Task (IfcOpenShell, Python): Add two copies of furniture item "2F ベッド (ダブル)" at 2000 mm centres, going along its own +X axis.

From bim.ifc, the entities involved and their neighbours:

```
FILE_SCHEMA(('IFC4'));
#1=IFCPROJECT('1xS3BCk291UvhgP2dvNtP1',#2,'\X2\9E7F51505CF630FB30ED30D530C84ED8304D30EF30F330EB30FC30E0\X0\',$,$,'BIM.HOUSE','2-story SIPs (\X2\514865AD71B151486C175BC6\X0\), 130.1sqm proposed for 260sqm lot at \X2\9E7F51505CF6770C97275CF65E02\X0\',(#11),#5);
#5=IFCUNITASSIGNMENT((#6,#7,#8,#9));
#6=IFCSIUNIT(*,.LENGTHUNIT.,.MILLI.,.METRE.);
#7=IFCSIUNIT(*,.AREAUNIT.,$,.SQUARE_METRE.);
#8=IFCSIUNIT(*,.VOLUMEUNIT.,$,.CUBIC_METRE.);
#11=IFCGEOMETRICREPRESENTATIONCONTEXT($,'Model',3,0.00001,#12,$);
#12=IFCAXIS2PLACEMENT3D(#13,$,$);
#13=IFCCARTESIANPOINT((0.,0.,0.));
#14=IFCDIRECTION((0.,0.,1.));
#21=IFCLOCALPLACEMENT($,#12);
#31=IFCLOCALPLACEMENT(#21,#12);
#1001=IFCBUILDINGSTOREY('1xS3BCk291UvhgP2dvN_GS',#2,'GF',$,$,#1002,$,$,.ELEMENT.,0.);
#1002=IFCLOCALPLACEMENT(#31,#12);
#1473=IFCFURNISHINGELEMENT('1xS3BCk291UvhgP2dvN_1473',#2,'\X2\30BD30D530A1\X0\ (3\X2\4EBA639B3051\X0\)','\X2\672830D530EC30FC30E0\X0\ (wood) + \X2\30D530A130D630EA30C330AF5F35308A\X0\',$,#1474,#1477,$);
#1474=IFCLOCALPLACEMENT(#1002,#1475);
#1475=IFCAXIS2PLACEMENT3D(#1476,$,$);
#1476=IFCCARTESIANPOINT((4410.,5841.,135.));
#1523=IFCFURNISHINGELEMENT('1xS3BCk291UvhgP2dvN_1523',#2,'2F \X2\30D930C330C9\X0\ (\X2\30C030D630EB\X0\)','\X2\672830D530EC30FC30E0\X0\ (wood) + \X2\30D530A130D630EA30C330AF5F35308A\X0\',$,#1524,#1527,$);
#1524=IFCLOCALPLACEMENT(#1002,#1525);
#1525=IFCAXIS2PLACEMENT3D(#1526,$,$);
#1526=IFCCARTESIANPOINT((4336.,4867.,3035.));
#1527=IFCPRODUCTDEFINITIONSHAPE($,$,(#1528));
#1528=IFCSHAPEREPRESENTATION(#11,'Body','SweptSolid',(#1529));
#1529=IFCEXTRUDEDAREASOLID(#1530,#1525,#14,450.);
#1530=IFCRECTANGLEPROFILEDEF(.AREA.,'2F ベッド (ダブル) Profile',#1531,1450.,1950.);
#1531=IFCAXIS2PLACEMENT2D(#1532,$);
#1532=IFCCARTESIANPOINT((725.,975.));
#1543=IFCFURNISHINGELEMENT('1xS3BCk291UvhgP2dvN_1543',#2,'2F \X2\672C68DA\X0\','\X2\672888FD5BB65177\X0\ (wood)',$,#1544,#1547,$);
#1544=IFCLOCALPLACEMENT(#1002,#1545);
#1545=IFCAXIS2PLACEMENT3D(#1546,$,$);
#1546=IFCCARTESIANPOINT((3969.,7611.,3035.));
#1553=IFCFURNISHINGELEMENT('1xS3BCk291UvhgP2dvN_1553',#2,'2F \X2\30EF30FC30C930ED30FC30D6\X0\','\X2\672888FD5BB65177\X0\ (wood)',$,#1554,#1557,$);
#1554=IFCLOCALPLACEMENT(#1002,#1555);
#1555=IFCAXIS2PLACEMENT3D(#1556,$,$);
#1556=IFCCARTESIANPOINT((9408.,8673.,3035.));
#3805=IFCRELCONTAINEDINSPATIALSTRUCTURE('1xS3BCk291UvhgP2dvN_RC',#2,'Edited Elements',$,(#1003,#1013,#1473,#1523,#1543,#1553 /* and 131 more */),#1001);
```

```python
import ifcopenshell
import ifcopenshell.api.geometry
import ifcopenshell.api.root
import ifcopenshell.util.element
import ifcopenshell.util.placement

model = ifcopenshell.open("bim.ifc")


def reuse_history(source, copy):
    """copy_class also copies each property set's owner history, people and application; keep the originals."""
    for rel in copy.IsDefinedBy:
        if rel.is_a("IfcRelDefinesByProperties") and (history := rel.RelatingPropertyDefinition.OwnerHistory):
            rel.RelatingPropertyDefinition.OwnerHistory = source.OwnerHistory
            ifcopenshell.util.element.remove_deep2(model, history)


source = model.by_id(1523)
base = ifcopenshell.util.placement.get_local_placement(source.ObjectPlacement)
step = base[:3, 0] * 2000.0

for i in range(1, 3):
    copy = ifcopenshell.api.root.copy_class(model, product=source)
    copy.Representation = ifcopenshell.util.element.copy_deep(
        model, source.Representation, exclude=["IfcGeometricRepresentationContext", "IfcRepresentationMap"]
    )
    reuse_history(source, copy)
    matrix = base.copy()
    matrix[:3, 3] += i * step
    print("added at", matrix[:3, 3].round(3) + 0.0)
    ifcopenshell.api.geometry.edit_object_placement(model, product=copy, matrix=matrix, is_si=False)

model.write("bim_edited.ifc")
```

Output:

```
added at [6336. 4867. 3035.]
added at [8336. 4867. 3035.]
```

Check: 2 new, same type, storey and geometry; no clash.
